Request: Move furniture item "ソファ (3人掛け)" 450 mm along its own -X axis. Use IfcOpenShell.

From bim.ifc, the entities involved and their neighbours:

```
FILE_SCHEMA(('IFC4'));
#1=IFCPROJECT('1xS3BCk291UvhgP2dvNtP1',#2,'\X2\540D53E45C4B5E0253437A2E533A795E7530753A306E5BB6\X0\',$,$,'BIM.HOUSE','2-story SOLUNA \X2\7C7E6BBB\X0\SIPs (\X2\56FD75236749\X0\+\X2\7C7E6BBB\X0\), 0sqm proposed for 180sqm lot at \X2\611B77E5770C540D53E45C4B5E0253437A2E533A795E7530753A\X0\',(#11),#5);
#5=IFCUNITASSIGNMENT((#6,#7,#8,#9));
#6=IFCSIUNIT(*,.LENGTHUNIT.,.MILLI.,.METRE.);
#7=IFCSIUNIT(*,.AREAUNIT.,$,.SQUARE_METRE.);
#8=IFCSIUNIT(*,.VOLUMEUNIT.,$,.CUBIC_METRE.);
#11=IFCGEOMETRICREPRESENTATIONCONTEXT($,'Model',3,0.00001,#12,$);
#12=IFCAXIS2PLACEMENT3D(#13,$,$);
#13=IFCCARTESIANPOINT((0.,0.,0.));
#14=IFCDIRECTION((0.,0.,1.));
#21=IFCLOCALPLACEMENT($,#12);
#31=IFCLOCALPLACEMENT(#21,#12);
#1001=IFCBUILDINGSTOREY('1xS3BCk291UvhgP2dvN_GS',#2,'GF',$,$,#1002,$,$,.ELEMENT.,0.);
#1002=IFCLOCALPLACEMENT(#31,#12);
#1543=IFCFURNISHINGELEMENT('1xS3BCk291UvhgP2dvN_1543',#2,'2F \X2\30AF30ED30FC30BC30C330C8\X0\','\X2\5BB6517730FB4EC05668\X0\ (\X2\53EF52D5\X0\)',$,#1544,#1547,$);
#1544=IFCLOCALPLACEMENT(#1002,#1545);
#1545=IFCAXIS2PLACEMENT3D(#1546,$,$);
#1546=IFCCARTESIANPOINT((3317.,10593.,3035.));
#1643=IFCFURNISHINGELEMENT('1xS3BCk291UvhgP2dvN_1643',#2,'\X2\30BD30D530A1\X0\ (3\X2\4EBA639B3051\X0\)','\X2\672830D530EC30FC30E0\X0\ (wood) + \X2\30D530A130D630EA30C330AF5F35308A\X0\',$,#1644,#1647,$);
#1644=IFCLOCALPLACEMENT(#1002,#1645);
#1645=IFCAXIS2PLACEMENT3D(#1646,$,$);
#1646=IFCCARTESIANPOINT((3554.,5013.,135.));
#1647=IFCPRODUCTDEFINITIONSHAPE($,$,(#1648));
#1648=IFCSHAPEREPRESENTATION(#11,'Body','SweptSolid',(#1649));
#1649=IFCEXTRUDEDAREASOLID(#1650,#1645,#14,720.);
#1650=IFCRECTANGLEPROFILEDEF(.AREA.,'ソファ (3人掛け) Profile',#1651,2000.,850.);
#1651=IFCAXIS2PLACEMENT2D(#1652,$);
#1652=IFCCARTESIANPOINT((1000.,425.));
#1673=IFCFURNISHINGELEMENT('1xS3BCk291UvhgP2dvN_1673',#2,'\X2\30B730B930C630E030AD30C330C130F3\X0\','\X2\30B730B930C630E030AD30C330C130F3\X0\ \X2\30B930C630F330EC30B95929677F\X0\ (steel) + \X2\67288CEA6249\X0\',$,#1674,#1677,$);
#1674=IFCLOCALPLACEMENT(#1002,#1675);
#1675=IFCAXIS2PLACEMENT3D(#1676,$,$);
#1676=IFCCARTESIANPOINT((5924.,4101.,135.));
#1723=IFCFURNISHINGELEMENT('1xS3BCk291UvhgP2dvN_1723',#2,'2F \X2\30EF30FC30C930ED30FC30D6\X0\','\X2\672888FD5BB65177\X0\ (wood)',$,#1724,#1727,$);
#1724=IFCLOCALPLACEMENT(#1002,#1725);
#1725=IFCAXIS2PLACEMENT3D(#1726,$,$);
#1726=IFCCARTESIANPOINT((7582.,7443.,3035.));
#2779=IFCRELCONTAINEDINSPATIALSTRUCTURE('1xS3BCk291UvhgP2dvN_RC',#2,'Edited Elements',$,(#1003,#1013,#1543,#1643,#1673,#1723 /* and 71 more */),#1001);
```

```python
import ifcopenshell
import ifcopenshell.api.geometry
import ifcopenshell.util.placement
import ifcopenshell.util.unit

model = ifcopenshell.open("bim.ifc")
unit_scale = ifcopenshell.util.unit.calculate_unit_scale(model)

item = model.by_guid("1xS3BCk291UvhgP2dvN_1643")
matrix = ifcopenshell.util.placement.get_local_placement(item.ObjectPlacement)
matrix[:3, 3] -= matrix[:3, 0] * 0.45 / unit_scale
ifcopenshell.api.geometry.edit_object_placement(model, product=item, matrix=matrix, is_si=False)

print(ifcopenshell.util.placement.get_local_placement(item.ObjectPlacement).round(3) + 0.0)

model.write("bim-out.ifc")
```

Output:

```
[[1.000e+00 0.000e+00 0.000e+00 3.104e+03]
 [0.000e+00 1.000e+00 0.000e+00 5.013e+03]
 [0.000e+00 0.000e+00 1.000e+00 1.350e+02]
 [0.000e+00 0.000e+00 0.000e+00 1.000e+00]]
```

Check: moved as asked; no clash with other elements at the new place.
